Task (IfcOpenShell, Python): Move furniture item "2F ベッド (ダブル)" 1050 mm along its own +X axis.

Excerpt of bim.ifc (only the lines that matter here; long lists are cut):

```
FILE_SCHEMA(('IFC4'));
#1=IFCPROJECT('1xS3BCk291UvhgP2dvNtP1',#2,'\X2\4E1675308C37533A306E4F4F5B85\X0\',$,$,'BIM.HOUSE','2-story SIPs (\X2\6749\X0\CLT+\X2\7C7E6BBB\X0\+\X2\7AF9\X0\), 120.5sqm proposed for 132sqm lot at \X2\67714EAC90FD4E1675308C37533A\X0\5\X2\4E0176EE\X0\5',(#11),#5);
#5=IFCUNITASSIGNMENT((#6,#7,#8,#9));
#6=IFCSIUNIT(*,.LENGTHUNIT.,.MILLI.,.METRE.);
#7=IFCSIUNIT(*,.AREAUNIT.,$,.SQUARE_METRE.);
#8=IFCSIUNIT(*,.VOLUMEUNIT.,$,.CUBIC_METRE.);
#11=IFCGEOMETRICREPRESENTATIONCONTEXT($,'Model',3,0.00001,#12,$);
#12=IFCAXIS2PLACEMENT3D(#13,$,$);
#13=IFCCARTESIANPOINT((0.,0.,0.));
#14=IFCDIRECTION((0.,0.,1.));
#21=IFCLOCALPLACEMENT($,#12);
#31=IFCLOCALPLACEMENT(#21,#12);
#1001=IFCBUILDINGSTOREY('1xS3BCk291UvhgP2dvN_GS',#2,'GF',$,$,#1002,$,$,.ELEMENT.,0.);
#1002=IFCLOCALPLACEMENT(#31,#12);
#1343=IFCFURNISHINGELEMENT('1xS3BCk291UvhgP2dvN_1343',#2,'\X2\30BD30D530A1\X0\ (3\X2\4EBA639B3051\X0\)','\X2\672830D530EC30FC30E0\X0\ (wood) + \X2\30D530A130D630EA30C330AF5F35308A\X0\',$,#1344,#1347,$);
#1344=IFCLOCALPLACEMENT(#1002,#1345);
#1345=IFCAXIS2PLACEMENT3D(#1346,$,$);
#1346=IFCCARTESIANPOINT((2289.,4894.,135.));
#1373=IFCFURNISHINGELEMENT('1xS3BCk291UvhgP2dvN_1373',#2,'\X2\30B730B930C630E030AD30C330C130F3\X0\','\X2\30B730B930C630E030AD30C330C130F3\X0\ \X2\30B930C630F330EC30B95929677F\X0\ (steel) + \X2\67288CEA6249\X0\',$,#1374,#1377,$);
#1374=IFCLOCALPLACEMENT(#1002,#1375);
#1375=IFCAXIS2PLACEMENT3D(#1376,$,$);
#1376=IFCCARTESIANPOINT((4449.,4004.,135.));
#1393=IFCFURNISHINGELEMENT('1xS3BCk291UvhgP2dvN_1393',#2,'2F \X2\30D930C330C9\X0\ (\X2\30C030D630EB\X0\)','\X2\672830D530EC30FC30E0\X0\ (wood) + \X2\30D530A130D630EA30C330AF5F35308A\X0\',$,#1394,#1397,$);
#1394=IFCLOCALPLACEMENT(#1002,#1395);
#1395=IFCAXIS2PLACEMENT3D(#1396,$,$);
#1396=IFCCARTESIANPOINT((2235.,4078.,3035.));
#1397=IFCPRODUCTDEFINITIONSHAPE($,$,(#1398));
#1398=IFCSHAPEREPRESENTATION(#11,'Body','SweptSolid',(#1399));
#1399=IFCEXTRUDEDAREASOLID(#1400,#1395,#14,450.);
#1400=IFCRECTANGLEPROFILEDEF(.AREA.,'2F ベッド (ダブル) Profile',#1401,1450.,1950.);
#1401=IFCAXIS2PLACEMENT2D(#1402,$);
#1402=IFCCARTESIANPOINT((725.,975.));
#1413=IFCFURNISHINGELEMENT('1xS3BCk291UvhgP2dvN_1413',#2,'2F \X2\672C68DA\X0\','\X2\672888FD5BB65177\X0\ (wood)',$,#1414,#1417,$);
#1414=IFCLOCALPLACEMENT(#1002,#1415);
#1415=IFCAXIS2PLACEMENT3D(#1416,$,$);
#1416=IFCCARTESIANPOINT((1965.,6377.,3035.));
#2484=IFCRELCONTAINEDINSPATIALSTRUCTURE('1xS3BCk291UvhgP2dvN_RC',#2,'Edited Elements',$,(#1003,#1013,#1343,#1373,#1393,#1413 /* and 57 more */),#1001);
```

```python
import ifcopenshell
import ifcopenshell.api.geometry
import ifcopenshell.util.placement
import ifcopenshell.util.unit

model = ifcopenshell.open("bim.ifc")
unit_scale = ifcopenshell.util.unit.calculate_unit_scale(model)

item = model.by_guid("1xS3BCk291UvhgP2dvN_1393")
matrix = ifcopenshell.util.placement.get_local_placement(item.ObjectPlacement)
matrix[:3, 3] += matrix[:3, 0] * 1.05 / unit_scale
ifcopenshell.api.geometry.edit_object_placement(model, product=item, matrix=matrix, is_si=False)

print(ifcopenshell.util.placement.get_local_placement(item.ObjectPlacement).round(3) + 0.0)

model.write("bim_v2.ifc")
```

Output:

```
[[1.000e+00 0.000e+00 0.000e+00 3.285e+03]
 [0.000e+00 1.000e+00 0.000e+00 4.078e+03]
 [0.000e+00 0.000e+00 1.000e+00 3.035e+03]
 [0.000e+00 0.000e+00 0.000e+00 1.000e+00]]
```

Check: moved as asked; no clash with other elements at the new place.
